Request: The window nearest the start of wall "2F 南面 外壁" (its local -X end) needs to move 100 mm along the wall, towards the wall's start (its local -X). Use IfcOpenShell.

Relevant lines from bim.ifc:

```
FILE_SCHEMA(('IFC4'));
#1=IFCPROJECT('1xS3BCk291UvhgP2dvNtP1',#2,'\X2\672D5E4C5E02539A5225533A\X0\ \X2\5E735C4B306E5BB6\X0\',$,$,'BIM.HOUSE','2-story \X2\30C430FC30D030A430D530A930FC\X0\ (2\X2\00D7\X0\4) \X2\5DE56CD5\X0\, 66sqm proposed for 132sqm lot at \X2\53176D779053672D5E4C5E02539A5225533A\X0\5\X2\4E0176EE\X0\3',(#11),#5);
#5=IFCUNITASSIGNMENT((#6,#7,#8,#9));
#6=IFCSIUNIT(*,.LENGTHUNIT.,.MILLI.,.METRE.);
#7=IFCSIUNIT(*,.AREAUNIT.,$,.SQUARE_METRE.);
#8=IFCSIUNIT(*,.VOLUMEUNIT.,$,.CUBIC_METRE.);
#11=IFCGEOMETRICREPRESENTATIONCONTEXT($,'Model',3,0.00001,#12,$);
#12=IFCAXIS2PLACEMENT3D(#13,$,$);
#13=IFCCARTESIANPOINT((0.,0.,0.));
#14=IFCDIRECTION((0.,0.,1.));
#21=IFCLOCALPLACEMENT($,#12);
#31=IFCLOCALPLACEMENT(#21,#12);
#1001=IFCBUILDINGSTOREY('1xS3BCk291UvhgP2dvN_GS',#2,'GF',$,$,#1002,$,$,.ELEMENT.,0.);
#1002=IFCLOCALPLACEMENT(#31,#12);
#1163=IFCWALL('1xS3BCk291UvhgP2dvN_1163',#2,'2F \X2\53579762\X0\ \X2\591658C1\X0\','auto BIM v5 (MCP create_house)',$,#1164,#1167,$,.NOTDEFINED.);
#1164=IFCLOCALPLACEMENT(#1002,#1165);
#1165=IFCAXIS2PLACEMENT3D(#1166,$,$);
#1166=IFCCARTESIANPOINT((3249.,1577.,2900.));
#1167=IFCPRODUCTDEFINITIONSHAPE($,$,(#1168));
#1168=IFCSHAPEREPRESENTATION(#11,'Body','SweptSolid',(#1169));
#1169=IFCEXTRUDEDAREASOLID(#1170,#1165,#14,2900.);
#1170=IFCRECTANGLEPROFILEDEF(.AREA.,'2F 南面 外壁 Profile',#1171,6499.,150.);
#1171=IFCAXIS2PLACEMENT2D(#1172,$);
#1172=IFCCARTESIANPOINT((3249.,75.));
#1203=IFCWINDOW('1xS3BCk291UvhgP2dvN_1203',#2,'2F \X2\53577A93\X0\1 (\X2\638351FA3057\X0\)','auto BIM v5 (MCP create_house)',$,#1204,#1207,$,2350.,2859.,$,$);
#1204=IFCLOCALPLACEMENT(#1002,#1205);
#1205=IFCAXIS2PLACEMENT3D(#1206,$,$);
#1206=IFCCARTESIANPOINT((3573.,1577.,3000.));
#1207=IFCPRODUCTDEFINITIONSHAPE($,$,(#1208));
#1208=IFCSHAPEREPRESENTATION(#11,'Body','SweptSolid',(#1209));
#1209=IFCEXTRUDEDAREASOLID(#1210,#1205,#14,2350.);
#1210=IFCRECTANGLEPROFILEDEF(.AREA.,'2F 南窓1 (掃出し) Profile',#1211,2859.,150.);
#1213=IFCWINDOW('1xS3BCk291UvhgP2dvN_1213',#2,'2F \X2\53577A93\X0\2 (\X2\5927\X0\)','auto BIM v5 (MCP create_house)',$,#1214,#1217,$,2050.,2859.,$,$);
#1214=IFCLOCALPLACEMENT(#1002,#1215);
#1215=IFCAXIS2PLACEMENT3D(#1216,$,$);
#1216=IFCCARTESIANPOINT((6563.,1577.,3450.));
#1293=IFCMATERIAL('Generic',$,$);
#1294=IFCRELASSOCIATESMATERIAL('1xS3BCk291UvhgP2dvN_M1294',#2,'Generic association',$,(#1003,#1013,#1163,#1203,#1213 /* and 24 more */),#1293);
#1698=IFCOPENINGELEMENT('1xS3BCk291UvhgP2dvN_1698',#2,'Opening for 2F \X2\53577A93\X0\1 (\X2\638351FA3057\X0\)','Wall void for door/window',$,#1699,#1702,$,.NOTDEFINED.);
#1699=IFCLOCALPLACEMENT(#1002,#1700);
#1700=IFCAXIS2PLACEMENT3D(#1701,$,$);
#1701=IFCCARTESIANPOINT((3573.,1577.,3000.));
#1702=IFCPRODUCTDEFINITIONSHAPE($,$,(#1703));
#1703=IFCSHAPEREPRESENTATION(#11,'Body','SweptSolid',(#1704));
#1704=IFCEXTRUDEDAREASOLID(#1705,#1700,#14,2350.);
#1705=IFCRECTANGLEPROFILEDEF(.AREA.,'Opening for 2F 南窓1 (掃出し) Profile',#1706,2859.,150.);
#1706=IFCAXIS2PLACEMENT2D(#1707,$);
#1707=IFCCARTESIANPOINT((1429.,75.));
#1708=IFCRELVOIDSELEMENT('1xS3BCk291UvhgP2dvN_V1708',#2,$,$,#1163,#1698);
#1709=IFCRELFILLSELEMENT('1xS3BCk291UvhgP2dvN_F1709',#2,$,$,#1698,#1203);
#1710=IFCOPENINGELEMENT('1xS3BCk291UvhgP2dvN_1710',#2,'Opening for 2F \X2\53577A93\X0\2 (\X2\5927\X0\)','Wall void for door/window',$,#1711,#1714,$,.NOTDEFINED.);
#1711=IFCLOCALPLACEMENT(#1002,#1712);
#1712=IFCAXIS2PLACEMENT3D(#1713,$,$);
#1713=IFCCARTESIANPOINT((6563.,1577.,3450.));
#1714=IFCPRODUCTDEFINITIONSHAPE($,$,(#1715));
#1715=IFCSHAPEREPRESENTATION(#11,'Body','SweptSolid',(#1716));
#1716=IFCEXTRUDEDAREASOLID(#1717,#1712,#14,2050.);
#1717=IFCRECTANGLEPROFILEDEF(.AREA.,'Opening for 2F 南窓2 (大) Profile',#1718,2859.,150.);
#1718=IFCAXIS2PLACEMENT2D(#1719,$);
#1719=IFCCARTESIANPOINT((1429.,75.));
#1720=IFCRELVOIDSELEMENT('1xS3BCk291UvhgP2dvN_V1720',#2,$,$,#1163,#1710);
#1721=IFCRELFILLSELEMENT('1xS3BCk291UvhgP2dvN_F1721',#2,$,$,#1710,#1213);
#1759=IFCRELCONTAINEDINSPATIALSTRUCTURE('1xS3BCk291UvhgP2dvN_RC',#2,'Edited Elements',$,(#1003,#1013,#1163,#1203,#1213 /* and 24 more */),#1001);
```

```python
import ifcopenshell
import ifcopenshell.api.geometry
import ifcopenshell.util.placement

model = ifcopenshell.open("bim.ifc")

window = model.by_guid("1xS3BCk291UvhgP2dvN_1203")
opening = window.FillsVoids[0].RelatingOpeningElement
wall = opening.VoidsElements[0].RelatingBuildingElement

wall_matrix = ifcopenshell.util.placement.get_local_placement(wall.ObjectPlacement)
shift = wall_matrix[:3, 0] * -100.0
before = ifcopenshell.util.placement.get_local_placement(window.ObjectPlacement)[:3, 3].copy()

# The window is not placed relative to its opening, so move both.
for product in (opening, window):
    matrix = ifcopenshell.util.placement.get_local_placement(product.ObjectPlacement)
    matrix[:3, 3] += shift
    ifcopenshell.api.geometry.edit_object_placement(model, product=product, matrix=matrix, is_si=False)

after = ifcopenshell.util.placement.get_local_placement(window.ObjectPlacement)[:3, 3]
print("window moved by", (after - before).round(3) + 0.0)

model.write("bim-out.ifc")
```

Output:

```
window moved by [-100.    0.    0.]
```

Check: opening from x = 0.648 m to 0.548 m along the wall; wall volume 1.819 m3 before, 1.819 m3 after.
